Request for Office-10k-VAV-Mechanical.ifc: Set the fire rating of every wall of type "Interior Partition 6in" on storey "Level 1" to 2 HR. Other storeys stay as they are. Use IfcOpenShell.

First a look at what the model holds.

```python
import ifcopenshell
import ifcopenshell.util.element

model = ifcopenshell.open("Office-10k-VAV-Mechanical.ifc")
print(model.schema)
storey = next(s for s in model.by_type("IfcBuildingStorey") if s.Name == "Level 1")
walls = [e for e in ifcopenshell.util.element.get_decomposition(storey) if e.is_a("IfcWall")]
seen = {}
for e in walls:
    element_type = ifcopenshell.util.element.get_type(e)
    key = (element_type.Name if element_type != e and element_type else None, ifcopenshell.util.element.get_pset(e, "Pset_WallCommon", "FireRating"))
    seen[key] = seen.get(key, 0) + 1
for (name, value), count in sorted(seen.items(), key=str):
    print(count, "x", name, "|", value)
```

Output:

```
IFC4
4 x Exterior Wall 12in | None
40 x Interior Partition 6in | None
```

```python
import ifcopenshell
import ifcopenshell.api.pset
import ifcopenshell.util.element

model = ifcopenshell.open("Office-10k-VAV-Mechanical.ifc")

storey = next(s for s in model.by_type("IfcBuildingStorey") if s.Name == "Level 1")
walls = [e for e in ifcopenshell.util.element.get_decomposition(storey) if e.is_a("IfcWall")]

count = 0
for e in walls:
    element_type = ifcopenshell.util.element.get_type(e)
    if element_type in (None, e) or element_type.Name != "Interior Partition 6in":
        continue
    # add_pset returns the element's existing set when there is one.
    pset = ifcopenshell.api.pset.add_pset(model, product=e, name="Pset_WallCommon")
    ifcopenshell.api.pset.edit_pset(model, pset=pset, properties={"FireRating": "2 HR"})
    count += 1

print(count, "walls updated")

model.write("Office-10k-VAV-Mechanical_rev.ifc")
```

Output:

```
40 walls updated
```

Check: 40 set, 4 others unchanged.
